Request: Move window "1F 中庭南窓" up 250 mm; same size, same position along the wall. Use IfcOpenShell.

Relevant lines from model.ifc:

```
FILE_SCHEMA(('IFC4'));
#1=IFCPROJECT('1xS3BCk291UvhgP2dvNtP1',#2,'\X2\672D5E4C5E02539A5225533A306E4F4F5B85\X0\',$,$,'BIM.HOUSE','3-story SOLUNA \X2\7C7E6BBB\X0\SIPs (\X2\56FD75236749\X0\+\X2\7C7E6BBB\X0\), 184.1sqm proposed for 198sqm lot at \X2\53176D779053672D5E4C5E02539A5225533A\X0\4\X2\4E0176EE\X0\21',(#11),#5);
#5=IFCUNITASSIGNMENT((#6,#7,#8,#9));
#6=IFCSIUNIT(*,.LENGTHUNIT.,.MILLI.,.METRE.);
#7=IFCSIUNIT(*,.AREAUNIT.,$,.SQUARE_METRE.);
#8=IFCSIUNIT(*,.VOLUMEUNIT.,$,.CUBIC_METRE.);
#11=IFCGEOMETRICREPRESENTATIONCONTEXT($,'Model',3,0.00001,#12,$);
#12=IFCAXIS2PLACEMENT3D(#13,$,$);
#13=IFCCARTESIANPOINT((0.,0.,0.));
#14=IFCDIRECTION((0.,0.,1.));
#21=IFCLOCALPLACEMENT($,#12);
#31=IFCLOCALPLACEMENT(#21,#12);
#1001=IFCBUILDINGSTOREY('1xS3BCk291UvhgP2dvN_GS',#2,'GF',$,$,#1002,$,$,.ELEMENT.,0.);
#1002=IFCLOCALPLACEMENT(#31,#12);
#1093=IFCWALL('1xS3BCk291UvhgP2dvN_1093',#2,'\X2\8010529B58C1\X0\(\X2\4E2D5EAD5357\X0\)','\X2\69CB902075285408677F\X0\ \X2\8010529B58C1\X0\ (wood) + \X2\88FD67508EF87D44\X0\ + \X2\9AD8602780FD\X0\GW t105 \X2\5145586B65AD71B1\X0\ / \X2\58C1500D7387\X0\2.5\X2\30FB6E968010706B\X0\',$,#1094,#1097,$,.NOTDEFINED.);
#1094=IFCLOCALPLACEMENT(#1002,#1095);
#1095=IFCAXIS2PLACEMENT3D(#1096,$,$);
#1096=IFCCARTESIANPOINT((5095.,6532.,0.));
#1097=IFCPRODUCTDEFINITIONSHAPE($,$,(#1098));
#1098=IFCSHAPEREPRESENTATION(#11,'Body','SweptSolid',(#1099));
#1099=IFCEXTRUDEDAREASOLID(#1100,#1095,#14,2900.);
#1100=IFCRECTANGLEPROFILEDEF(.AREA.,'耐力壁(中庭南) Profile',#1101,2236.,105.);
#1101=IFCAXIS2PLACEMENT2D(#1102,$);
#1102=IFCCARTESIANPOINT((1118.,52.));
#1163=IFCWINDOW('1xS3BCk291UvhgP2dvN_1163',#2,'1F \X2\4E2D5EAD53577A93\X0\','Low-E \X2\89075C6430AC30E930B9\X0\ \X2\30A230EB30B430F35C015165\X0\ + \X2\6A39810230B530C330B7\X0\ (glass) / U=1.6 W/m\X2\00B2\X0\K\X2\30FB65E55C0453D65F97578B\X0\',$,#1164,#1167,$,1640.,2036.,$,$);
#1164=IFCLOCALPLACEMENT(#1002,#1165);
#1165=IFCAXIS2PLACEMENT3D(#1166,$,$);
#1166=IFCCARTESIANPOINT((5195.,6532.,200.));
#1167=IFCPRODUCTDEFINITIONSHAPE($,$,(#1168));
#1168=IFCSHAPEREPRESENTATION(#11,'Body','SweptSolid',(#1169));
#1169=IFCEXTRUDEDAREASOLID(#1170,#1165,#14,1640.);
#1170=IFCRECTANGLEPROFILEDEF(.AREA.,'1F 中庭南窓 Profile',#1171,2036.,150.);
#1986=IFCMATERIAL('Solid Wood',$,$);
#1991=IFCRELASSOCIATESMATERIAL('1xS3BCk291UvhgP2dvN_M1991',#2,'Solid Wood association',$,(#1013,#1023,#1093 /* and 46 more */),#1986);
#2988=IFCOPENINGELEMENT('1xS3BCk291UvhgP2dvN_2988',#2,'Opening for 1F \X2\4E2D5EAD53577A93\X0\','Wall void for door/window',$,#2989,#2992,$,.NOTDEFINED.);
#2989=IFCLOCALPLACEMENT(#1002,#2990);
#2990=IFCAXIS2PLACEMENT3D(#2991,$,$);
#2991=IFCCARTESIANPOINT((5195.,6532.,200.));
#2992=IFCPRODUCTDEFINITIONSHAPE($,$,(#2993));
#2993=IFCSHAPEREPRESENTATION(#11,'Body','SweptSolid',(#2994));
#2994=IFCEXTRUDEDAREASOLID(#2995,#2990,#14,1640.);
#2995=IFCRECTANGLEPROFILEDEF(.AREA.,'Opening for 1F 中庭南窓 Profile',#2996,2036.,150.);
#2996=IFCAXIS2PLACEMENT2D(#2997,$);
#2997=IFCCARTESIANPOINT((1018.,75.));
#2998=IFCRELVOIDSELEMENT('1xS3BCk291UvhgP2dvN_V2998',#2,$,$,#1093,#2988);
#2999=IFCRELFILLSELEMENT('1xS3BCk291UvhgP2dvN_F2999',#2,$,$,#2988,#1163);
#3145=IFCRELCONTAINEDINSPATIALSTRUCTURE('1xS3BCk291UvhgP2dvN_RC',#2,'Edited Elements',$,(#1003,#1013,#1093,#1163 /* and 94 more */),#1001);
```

```python
import numpy as np
import ifcopenshell
import ifcopenshell.api.geometry
import ifcopenshell.util.placement
import ifcopenshell.util.unit

model = ifcopenshell.open("model.ifc")
unit_scale = ifcopenshell.util.unit.calculate_unit_scale(model)

window = model.by_id(1163)
opening = window.FillsVoids[0].RelatingOpeningElement
dz = 0.25 / unit_scale

shift = np.array([0.0, 0.0, dz])
# The window is not placed relative to its opening, so move both.
for product in (opening, window):
    matrix = ifcopenshell.util.placement.get_local_placement(product.ObjectPlacement)
    matrix[:3, 3] += shift
    ifcopenshell.api.geometry.edit_object_placement(model, product=product, matrix=matrix, is_si=False)

print(f"moved by {dz * unit_scale:+.3f} m")

model.write("model_edited.ifc")
```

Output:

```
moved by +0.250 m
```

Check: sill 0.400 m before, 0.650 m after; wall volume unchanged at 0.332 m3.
